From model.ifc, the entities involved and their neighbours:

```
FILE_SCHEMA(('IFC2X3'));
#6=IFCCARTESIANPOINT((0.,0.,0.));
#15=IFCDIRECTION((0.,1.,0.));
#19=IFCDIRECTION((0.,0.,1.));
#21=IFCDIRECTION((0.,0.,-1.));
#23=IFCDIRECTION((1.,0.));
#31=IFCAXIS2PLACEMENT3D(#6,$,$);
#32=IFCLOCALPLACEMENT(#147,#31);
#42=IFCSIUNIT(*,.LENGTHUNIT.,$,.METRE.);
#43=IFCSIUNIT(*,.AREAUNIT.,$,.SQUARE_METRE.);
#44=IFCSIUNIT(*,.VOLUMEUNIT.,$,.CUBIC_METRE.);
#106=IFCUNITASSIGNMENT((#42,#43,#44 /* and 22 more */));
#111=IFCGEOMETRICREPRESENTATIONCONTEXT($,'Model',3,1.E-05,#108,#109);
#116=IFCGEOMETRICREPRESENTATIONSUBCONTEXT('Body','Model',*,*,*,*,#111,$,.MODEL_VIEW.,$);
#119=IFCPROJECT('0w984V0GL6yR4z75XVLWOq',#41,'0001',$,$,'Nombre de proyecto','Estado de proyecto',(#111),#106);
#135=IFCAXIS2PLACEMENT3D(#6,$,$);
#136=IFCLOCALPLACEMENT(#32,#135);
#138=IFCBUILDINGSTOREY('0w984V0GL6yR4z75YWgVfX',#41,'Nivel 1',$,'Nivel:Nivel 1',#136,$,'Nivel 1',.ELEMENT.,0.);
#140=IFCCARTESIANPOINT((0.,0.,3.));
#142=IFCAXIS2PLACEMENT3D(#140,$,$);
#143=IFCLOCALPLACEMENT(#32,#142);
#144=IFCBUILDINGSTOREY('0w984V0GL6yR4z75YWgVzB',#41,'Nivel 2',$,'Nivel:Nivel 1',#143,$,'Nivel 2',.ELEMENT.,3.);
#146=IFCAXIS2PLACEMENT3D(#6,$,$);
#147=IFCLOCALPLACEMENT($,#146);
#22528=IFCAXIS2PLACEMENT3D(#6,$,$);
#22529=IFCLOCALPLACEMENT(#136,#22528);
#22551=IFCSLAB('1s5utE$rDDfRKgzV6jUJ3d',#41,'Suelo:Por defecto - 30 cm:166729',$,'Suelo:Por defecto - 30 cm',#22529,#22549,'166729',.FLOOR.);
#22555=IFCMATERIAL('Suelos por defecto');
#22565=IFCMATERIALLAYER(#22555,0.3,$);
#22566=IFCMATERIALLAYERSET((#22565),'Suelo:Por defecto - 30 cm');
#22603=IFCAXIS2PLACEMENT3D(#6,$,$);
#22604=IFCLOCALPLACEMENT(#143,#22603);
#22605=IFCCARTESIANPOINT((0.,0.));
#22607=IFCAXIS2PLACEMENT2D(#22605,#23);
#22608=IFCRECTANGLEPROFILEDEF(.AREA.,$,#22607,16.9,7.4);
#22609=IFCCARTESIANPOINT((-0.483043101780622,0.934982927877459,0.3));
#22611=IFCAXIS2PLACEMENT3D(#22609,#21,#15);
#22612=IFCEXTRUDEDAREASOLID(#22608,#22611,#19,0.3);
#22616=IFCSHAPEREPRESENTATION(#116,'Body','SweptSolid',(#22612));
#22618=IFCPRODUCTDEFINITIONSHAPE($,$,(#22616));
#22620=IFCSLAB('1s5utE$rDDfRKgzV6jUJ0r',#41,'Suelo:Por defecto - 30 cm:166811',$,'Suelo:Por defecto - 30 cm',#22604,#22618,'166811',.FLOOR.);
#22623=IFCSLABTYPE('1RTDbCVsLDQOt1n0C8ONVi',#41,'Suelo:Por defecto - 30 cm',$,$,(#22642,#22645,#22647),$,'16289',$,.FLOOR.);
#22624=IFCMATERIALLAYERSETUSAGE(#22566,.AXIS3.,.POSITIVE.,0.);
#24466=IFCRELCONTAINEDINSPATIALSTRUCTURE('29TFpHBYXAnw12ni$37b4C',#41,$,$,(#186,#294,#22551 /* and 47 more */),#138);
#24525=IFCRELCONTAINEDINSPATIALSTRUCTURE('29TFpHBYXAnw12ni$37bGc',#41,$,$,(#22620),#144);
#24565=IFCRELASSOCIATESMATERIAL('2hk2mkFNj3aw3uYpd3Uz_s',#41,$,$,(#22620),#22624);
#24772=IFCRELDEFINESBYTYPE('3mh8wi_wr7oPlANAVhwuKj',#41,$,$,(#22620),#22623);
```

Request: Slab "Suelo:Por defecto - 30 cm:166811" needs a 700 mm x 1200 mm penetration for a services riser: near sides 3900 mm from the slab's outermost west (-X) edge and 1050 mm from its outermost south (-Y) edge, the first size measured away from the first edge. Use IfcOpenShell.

```python
import numpy as np
import ifcopenshell
import ifcopenshell.api.feature
import ifcopenshell.api.geometry
import ifcopenshell.api.root
import ifcopenshell.geom
import ifcopenshell.util.placement
import ifcopenshell.util.representation
import ifcopenshell.util.shape
import ifcopenshell.util.unit

model = ifcopenshell.open("model.ifc")
unit_scale = ifcopenshell.util.unit.calculate_unit_scale(model)
settings = ifcopenshell.geom.settings()


def volume(element):
    """Net volume in cubic metres, openings subtracted."""
    shape = ifcopenshell.geom.create_shape(settings, element)
    return ifcopenshell.util.shape.get_volume(shape.geometry)


slab = model.by_guid("1s5utE$rDDfRKgzV6jUJ0r")
before = volume(slab)

# Extent in the slab's own axes, in metres. The edges named are its -X and -Y sides.
slab_shape = ifcopenshell.geom.create_shape(settings, slab)
vertices = ifcopenshell.util.shape.get_vertices(slab_shape.geometry)
x_min, y_min, bottom = vertices.min(axis=0)
top = vertices[:, 2].max()

opening = ifcopenshell.api.root.create_entity(model, ifc_class="IfcOpeningElement", name="Services riser opening")
context = ifcopenshell.util.representation.get_context(model, "Model", "Body", "MODEL_VIEW")
width, depth = 0.7, 1.2
outline = [(0.0, 0.0), (width, 0.0), (width, depth), (0.0, depth), (0.0, 0.0)]
# Overshoot both faces by 50 mm so the cut is clean.
shape = ifcopenshell.api.geometry.add_slab_representation(
    model, context=context, depth=top - bottom + 0.1, polyline=outline
)
ifcopenshell.api.geometry.assign_representation(model, product=opening, representation=shape)

matrix = ifcopenshell.util.placement.get_local_placement(slab.ObjectPlacement)
matrix[:, 3] = matrix @ np.append(np.array([x_min + 3.9, y_min + 1.05, bottom - 0.05]) / unit_scale, 1.0)
ifcopenshell.api.geometry.edit_object_placement(model, product=opening, matrix=matrix, is_si=False)
ifcopenshell.api.feature.add_feature(model, feature=opening, element=slab)

after = volume(slab)

print(f"slab volume {before:.3f} -> {after:.3f} m3")

model.write("model-out.ifc")
```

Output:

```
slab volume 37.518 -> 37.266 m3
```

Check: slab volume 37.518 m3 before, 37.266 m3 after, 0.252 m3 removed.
